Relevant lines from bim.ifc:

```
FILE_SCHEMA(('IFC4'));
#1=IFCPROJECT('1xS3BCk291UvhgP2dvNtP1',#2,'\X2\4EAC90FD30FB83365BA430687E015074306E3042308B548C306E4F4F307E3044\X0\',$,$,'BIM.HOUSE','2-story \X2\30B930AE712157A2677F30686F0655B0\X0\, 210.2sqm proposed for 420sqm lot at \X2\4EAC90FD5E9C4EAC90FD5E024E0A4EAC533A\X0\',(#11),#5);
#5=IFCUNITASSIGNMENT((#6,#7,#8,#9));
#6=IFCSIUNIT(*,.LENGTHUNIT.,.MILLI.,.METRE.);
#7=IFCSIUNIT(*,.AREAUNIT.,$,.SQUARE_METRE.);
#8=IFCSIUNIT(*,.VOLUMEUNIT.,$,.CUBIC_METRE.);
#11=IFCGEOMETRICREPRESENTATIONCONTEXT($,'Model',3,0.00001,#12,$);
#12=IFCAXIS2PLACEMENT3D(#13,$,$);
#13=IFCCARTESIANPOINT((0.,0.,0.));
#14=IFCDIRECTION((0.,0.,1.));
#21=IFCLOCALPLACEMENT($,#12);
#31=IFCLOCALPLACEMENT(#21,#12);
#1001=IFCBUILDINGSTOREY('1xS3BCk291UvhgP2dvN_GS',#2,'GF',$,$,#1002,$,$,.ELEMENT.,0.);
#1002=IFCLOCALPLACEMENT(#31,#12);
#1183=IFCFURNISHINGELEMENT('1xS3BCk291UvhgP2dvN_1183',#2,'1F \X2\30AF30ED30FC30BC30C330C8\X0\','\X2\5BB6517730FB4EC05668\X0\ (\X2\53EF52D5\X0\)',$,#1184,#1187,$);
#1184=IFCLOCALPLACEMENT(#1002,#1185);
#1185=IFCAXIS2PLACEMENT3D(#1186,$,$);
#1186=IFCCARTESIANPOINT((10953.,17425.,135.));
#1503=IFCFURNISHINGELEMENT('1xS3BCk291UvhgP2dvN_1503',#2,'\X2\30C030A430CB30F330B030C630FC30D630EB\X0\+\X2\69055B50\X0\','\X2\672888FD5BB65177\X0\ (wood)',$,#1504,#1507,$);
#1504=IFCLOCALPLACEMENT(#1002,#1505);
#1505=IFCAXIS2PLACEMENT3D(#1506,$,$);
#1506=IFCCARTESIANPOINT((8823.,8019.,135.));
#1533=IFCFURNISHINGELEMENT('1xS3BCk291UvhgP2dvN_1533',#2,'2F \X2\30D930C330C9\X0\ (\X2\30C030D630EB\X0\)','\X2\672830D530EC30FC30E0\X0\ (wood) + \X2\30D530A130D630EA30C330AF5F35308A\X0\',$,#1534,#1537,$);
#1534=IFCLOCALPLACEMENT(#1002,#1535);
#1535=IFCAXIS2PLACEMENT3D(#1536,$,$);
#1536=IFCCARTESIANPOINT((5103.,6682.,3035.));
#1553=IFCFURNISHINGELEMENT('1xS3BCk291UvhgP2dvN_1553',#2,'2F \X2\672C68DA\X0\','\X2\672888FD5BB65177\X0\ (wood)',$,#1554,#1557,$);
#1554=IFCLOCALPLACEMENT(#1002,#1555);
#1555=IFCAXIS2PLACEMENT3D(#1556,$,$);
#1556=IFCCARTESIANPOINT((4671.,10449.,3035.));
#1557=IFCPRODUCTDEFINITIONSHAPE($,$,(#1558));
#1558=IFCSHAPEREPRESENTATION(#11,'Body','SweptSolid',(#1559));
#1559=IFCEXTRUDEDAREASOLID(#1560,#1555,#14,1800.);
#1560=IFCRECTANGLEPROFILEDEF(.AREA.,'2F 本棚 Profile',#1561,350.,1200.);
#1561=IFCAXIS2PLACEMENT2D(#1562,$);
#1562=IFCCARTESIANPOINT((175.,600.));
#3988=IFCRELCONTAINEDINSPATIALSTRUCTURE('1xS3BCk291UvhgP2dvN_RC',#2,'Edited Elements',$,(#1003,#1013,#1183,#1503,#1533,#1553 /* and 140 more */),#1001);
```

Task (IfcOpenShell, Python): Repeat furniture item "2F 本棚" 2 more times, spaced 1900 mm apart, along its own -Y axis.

```python
import ifcopenshell
import ifcopenshell.api.geometry
import ifcopenshell.api.root
import ifcopenshell.util.element
import ifcopenshell.util.placement

model = ifcopenshell.open("bim.ifc")


def reuse_history(source, copy):
    """copy_class also copies each property set's owner history, people and application; keep the originals."""
    for rel in copy.IsDefinedBy:
        if rel.is_a("IfcRelDefinesByProperties") and (history := rel.RelatingPropertyDefinition.OwnerHistory):
            rel.RelatingPropertyDefinition.OwnerHistory = source.OwnerHistory
            ifcopenshell.util.element.remove_deep2(model, history)


source = model.by_guid("1xS3BCk291UvhgP2dvN_1553")
base = ifcopenshell.util.placement.get_local_placement(source.ObjectPlacement)
step = -base[:3, 1] * 1900.0

for i in range(1, 3):
    copy = ifcopenshell.api.root.copy_class(model, product=source)
    copy.Representation = ifcopenshell.util.element.copy_deep(
        model, source.Representation, exclude=["IfcGeometricRepresentationContext", "IfcRepresentationMap"]
    )
    reuse_history(source, copy)
    matrix = base.copy()
    matrix[:3, 3] += i * step
    print("added at", matrix[:3, 3].round(3) + 0.0)
    ifcopenshell.api.geometry.edit_object_placement(model, product=copy, matrix=matrix, is_si=False)

model.write("bim_v2.ifc")
```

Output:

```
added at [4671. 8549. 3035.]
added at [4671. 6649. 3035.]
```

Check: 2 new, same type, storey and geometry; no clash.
